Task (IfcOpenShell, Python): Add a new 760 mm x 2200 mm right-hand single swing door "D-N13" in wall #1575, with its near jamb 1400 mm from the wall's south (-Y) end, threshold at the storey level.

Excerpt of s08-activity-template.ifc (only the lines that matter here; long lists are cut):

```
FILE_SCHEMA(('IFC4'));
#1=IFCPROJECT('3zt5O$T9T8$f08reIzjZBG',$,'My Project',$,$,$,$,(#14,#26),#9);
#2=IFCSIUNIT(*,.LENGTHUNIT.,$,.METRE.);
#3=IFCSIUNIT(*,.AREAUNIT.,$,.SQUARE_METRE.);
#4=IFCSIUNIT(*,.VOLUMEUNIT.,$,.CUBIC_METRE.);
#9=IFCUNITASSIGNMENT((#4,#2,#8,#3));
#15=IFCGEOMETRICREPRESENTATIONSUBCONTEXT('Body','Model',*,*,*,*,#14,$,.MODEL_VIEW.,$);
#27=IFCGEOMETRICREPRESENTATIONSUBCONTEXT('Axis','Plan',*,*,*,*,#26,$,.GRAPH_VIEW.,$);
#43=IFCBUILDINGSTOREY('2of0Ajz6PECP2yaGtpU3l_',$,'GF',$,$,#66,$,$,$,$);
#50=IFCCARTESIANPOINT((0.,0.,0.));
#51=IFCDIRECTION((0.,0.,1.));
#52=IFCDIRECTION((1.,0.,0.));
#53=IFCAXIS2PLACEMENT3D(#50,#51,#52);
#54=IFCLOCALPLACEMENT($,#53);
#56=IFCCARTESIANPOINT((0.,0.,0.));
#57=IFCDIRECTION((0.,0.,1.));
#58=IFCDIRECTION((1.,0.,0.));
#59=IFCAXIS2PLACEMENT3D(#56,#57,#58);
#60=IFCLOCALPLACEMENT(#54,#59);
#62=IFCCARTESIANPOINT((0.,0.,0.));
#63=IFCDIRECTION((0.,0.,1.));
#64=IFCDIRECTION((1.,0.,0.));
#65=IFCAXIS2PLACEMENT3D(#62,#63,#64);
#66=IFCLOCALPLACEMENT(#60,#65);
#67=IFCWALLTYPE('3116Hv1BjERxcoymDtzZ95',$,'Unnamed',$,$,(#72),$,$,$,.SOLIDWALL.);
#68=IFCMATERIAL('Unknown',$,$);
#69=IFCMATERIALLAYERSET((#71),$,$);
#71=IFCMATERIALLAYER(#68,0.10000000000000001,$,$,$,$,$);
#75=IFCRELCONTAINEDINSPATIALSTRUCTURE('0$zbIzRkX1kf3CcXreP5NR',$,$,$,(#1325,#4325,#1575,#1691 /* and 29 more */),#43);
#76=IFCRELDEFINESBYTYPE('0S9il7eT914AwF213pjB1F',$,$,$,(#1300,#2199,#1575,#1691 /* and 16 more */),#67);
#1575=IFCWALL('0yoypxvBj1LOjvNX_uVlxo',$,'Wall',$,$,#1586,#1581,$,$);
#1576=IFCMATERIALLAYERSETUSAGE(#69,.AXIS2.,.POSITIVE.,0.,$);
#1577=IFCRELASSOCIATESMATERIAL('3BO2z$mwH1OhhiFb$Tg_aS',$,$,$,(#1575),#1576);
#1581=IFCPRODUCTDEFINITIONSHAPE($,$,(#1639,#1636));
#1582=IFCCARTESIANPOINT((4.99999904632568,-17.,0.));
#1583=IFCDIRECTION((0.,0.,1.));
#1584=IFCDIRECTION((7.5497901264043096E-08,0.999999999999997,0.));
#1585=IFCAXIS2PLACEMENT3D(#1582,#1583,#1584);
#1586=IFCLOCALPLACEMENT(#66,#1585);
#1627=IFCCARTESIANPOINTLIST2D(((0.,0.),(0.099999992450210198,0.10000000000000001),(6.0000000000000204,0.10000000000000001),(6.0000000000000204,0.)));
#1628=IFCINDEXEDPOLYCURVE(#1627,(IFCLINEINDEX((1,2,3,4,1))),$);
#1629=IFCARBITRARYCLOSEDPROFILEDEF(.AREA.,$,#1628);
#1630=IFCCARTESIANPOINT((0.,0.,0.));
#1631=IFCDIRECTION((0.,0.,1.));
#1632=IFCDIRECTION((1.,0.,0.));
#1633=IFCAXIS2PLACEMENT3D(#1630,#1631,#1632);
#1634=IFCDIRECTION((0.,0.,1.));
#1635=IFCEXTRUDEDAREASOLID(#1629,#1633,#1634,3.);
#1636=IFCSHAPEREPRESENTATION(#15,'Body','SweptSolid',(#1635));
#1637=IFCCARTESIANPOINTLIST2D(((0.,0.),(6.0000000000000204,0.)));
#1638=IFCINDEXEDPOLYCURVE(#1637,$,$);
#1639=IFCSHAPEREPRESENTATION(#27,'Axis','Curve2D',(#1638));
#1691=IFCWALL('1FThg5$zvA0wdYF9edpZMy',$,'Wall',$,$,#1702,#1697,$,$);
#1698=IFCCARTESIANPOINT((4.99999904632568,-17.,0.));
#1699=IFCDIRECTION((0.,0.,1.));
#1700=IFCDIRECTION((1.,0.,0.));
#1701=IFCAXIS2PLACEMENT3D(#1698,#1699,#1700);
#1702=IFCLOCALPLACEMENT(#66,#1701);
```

```python
import numpy as np
import ifcopenshell
import ifcopenshell.api.feature
import ifcopenshell.api.geometry
import ifcopenshell.api.root
import ifcopenshell.api.spatial
import ifcopenshell.geom
import ifcopenshell.util.element
import ifcopenshell.util.placement
import ifcopenshell.util.representation
import ifcopenshell.util.shape
import ifcopenshell.util.unit

model = ifcopenshell.open("s08-activity-template.ifc")
unit_scale = ifcopenshell.util.unit.calculate_unit_scale(model)
settings = ifcopenshell.geom.settings()


def volume(element):
    """Net volume in cubic metres, openings subtracted."""
    shape = ifcopenshell.geom.create_shape(settings, element)
    return ifcopenshell.util.shape.get_volume(shape.geometry)


wall = model.by_guid("0yoypxvBj1LOjvNX_uVlxo")
storey = ifcopenshell.util.element.get_container(wall, ifc_class="IfcBuildingStorey")
context = ifcopenshell.util.representation.get_context(model, "Model", "Body", "MODEL_VIEW")
before = volume(wall)

width, height, from_end, sill = 0.76, 2.2, 1.4, 0.0  # metres

# The wall runs along its own X axis, and the end named is its -X end.
wall_shape = ifcopenshell.geom.create_shape(settings, wall)
x, y, z = ifcopenshell.util.shape.get_vertices(wall_shape.geometry).T
start = x.min() + from_end
face, thickness = float(y.min()), float(y.max() - y.min())
wall_matrix = ifcopenshell.util.placement.get_local_placement(wall.ObjectPlacement)
level = ifcopenshell.util.placement.get_local_placement(storey.ObjectPlacement)[2, 3]


def in_wall(x, y):
    """Placement at x, y metres in the wall's axes, at sill height."""
    matrix = wall_matrix.copy()
    matrix[:, 3] = wall_matrix @ np.array([x / unit_scale, y / unit_scale, 0.0, 1.0])
    matrix[2, 3] = level + sill / unit_scale
    return matrix


# Opening: a box that overshoots both wall faces by 50 mm.
opening = ifcopenshell.api.root.create_entity(model, ifc_class="IfcOpeningElement", predefined_type="OPENING")
box = ifcopenshell.api.geometry.add_wall_representation(
    model, context=context, length=width, height=height, thickness=thickness + 0.1
)
ifcopenshell.api.geometry.assign_representation(model, product=opening, representation=box)
ifcopenshell.api.geometry.edit_object_placement(model, product=opening, matrix=in_wall(start, face - 0.05), is_si=False)
ifcopenshell.api.feature.add_feature(model, feature=opening, element=wall)

door = ifcopenshell.api.root.create_entity(model, ifc_class="IfcDoor", name="D-N13", predefined_type="DOOR")
door.OverallWidth, door.OverallHeight = width / unit_scale, height / unit_scale
door.OperationType = "SINGLE_SWING_RIGHT"
body = ifcopenshell.api.geometry.add_door_representation(
    model,
    context=context,
    overall_width=door.OverallWidth,
    overall_height=door.OverallHeight,
    operation_type="SINGLE_SWING_RIGHT",
    lining_properties={"LiningDepth": thickness / unit_scale, "ThresholdDepth": thickness / unit_scale},
)
ifcopenshell.api.geometry.assign_representation(model, product=door, representation=body)
ifcopenshell.api.spatial.assign_container(model, products=[door], relating_structure=storey)
ifcopenshell.api.feature.add_filling(model, opening=opening, element=door)

# The lining spans the wall, so the door starts at the wall face.
ifcopenshell.api.geometry.edit_object_placement(model, product=door, matrix=in_wall(start, face), is_si=False)

after = volume(wall)

print(f"wall volume {before:.3f} -> {after:.3f} m3")

model.write("s08-activity-template_v2.ifc")
```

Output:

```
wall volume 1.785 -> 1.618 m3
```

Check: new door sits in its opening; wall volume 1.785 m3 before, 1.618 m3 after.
